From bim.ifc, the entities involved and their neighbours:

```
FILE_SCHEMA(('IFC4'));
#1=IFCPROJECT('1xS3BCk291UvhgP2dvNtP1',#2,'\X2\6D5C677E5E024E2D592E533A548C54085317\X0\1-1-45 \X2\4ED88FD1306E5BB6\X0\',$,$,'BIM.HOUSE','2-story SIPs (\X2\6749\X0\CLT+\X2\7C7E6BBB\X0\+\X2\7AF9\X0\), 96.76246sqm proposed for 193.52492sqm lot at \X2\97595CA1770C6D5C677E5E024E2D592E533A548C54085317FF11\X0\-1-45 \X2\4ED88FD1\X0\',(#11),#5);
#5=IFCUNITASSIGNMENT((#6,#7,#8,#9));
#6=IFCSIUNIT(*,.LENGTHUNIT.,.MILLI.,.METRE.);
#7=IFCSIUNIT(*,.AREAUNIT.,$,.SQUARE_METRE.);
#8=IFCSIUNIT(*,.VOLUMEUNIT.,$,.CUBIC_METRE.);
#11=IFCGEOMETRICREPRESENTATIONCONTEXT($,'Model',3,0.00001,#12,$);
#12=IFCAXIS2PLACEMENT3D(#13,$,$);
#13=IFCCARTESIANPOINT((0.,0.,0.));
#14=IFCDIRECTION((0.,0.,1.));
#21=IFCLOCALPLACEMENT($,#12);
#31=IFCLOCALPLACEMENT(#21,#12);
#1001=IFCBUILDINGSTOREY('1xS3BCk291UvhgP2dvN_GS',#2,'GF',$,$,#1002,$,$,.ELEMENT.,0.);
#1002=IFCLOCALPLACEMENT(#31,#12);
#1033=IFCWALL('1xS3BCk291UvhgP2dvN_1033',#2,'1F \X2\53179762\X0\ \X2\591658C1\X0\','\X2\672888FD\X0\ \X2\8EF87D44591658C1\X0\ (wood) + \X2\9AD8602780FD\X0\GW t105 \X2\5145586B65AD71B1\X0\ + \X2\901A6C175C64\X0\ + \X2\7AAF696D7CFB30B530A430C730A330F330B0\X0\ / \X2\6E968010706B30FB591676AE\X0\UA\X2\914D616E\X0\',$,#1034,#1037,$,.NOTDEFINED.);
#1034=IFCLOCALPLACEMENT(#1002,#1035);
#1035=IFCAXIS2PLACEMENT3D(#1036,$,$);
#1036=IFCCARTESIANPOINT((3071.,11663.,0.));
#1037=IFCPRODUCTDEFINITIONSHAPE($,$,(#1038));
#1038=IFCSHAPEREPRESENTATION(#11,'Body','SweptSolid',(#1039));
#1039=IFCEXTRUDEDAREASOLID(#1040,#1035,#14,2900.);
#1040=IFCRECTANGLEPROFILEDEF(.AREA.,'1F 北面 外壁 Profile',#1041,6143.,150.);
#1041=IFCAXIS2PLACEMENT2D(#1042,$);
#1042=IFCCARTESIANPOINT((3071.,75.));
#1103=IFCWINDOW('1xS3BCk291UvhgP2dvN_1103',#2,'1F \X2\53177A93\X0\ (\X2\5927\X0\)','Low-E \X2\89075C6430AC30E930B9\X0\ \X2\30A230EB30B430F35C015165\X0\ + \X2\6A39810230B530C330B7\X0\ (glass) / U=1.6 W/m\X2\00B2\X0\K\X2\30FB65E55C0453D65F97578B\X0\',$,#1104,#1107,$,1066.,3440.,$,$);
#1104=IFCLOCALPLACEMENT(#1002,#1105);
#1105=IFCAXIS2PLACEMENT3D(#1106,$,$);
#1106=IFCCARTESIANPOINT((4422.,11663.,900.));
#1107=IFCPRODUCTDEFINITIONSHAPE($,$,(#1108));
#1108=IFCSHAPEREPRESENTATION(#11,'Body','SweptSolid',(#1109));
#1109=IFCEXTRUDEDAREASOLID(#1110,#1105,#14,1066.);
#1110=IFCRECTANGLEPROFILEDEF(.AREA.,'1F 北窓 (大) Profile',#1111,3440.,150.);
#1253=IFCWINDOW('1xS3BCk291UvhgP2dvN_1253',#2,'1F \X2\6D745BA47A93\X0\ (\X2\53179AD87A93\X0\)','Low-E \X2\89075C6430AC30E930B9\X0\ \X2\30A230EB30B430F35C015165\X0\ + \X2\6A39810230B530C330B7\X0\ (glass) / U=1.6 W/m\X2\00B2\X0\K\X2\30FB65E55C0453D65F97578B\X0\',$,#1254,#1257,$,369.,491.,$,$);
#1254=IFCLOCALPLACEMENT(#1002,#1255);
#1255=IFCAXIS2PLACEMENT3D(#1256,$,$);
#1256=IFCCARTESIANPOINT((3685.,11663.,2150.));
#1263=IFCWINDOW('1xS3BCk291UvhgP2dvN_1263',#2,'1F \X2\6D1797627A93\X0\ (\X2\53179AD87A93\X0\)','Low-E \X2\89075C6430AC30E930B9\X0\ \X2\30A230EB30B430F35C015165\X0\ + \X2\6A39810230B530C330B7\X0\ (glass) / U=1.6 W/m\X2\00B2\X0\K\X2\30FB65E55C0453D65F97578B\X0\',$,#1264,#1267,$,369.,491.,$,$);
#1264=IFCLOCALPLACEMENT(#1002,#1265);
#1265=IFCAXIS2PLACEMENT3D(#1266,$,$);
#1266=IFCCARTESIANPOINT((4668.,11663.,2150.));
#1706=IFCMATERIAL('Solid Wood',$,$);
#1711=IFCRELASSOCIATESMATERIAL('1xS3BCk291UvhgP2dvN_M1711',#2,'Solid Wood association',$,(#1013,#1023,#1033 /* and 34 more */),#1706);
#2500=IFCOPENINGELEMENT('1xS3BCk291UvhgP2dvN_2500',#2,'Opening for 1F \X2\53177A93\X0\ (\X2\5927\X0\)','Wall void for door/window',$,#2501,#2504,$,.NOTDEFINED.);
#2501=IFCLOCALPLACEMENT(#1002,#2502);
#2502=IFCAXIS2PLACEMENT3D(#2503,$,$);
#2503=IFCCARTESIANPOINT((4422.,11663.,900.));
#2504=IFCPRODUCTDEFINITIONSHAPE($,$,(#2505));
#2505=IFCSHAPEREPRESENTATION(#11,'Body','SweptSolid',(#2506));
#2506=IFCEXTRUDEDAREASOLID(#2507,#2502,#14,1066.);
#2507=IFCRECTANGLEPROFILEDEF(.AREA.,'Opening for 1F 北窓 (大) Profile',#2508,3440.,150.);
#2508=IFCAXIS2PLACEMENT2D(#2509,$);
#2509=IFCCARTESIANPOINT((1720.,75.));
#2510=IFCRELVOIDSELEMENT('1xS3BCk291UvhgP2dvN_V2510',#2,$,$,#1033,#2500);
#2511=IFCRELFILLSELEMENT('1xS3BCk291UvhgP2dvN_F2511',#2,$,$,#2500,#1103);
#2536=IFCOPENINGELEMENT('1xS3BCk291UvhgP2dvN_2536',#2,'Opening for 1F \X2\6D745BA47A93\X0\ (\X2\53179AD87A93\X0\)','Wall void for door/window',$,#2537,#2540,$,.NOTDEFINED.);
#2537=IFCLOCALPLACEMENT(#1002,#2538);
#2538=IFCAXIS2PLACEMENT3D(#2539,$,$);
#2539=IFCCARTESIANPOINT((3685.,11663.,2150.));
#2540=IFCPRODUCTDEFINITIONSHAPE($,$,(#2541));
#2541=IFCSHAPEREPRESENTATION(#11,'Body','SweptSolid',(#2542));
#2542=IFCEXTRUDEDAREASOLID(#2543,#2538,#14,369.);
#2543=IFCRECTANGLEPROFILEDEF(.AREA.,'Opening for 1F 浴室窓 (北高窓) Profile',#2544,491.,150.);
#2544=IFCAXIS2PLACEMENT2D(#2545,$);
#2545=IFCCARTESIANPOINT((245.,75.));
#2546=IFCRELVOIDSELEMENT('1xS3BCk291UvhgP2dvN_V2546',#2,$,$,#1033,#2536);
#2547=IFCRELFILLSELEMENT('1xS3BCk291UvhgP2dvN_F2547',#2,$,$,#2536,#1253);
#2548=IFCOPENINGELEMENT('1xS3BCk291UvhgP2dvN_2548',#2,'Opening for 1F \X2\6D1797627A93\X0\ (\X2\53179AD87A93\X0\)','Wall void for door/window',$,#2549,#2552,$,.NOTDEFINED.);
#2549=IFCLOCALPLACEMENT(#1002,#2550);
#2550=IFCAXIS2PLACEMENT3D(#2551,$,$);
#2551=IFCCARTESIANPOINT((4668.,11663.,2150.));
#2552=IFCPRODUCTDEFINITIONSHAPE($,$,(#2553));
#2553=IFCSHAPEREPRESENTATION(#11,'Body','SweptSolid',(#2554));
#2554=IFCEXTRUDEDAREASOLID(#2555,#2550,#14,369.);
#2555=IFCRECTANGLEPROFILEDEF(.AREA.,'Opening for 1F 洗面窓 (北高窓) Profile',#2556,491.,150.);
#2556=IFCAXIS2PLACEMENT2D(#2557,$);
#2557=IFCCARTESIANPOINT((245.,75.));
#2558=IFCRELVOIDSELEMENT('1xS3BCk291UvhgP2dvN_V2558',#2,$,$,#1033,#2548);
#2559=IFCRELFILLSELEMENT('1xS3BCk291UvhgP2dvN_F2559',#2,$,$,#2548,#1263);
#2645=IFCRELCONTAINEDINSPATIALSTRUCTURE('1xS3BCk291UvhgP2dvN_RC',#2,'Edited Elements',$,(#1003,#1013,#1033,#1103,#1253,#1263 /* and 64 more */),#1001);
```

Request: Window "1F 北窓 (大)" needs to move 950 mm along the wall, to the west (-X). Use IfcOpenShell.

```python
import ifcopenshell
import ifcopenshell.api.geometry
import ifcopenshell.util.placement

model = ifcopenshell.open("bim.ifc")

window = model.by_guid("1xS3BCk291UvhgP2dvN_1103")
opening = window.FillsVoids[0].RelatingOpeningElement
wall = opening.VoidsElements[0].RelatingBuildingElement

wall_matrix = ifcopenshell.util.placement.get_local_placement(wall.ObjectPlacement)
shift = wall_matrix[:3, 0] * -950.0
before = ifcopenshell.util.placement.get_local_placement(window.ObjectPlacement)[:3, 3].copy()

# The window is not placed relative to its opening, so move both.
for product in (opening, window):
    matrix = ifcopenshell.util.placement.get_local_placement(product.ObjectPlacement)
    matrix[:3, 3] += shift
    ifcopenshell.api.geometry.edit_object_placement(model, product=product, matrix=matrix, is_si=False)

after = ifcopenshell.util.placement.get_local_placement(window.ObjectPlacement)[:3, 3]
print("window moved by", (after - before).round(3) + 0.0)

model.write("bim_v2.ifc")
```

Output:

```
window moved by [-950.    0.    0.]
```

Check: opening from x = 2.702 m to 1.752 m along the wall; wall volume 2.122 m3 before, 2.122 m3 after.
